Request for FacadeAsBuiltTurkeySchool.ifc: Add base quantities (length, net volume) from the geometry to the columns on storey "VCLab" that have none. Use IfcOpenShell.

First a look at what the model holds.

```python
import ifcopenshell
import ifcopenshell.util.element
import ifcopenshell.util.unit

model = ifcopenshell.open("FacadeAsBuiltTurkeySchool.ifc")
print(model.schema)
for unit_type in ("LENGTHUNIT", "AREAUNIT", "VOLUMEUNIT"):
    print(unit_type, ifcopenshell.util.unit.calculate_unit_scale(model, unit_type))
storey = next(s for s in model.by_type("IfcBuildingStorey") if s.Name == "VCLab")
columns = [e for e in ifcopenshell.util.element.get_decomposition(storey) if e.is_a("IfcColumn")]
for e in sorted(columns, key=lambda e: e.id()):
    print(e.id(), e.is_a(), e.Name, list(ifcopenshell.util.element.get_psets(e, qtos_only=True)), sep=" | ")
```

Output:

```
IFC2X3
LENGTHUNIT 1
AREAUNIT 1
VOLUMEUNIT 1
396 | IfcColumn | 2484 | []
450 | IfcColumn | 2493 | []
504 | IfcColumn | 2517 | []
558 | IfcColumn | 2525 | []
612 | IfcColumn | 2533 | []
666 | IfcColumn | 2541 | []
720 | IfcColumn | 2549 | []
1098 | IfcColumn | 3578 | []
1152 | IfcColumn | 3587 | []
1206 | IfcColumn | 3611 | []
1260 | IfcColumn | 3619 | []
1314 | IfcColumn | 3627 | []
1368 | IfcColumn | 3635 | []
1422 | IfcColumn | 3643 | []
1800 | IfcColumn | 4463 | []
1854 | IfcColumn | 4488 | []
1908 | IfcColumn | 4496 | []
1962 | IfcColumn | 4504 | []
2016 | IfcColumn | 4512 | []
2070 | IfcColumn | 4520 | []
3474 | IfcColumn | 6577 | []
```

```python
import ifcopenshell
import ifcopenshell.api.pset
import ifcopenshell.geom
import ifcopenshell.util.element
import ifcopenshell.util.shape
import ifcopenshell.util.unit

model = ifcopenshell.open("FacadeAsBuiltTurkeySchool.ifc")
unit_scale = ifcopenshell.util.unit.calculate_unit_scale(model)
volume_scale = ifcopenshell.util.unit.calculate_unit_scale(model, "VOLUMEUNIT")
settings = ifcopenshell.geom.settings()

storey = next(s for s in model.by_type("IfcBuildingStorey") if s.Name == "VCLab")
columns = [e for e in ifcopenshell.util.element.get_decomposition(storey) if e.is_a("IfcColumn")]

for e in sorted(columns, key=lambda e: e.id()):
    if ifcopenshell.util.element.get_psets(e, qtos_only=True, should_inherit=False):
        continue
    # Geometry comes back in metres, in the element's own axes.
    shape = ifcopenshell.geom.create_shape(settings, e)
    values = {
        "Length": ifcopenshell.util.shape.get_z(shape.geometry) / unit_scale,
        "NetVolume": ifcopenshell.util.shape.get_volume(shape.geometry) / volume_scale,
    }
    qto = ifcopenshell.api.pset.add_qto(model, product=e, name="BaseQuantities")
    ifcopenshell.api.pset.edit_qto(model, qto=qto, properties=values)
    print(e.id(), {k: round(v, 3) for k, v in values.items()})

model.write("FacadeAsBuiltTurkeySchool_rev.ifc")
```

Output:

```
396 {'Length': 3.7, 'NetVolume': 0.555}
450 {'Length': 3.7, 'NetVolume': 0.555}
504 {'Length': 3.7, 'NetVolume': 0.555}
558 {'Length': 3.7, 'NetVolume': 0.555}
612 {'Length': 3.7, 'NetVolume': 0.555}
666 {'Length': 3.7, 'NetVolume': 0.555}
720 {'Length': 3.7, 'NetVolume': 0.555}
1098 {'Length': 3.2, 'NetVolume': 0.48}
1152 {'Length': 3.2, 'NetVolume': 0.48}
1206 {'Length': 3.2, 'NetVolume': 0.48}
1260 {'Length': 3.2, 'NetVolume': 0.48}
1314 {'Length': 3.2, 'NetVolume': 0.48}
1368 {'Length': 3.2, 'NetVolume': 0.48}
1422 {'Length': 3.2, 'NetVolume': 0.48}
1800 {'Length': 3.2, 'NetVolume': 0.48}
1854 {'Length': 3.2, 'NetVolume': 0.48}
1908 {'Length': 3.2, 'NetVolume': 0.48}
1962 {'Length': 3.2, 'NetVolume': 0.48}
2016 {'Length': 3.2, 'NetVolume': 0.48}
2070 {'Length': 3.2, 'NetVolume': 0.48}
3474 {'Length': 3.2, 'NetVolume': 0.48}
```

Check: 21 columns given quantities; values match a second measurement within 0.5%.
